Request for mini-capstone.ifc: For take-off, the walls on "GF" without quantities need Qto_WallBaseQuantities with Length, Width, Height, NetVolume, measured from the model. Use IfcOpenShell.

First a look at what the model holds.

```python
import ifcopenshell
import ifcopenshell.util.element
import ifcopenshell.util.unit

model = ifcopenshell.open("mini-capstone.ifc")
print(model.schema)
for unit_type in ("LENGTHUNIT", "AREAUNIT", "VOLUMEUNIT"):
    print(unit_type, ifcopenshell.util.unit.calculate_unit_scale(model, unit_type))
storey = next(s for s in model.by_type("IfcBuildingStorey") if s.Name == "GF")
walls = [e for e in ifcopenshell.util.element.get_decomposition(storey) if e.is_a("IfcWall")]
for e in sorted(walls, key=lambda e: e.id()):
    print(e.id(), e.is_a(), e.Name, list(ifcopenshell.util.element.get_psets(e, qtos_only=True)), sep=" | ")
```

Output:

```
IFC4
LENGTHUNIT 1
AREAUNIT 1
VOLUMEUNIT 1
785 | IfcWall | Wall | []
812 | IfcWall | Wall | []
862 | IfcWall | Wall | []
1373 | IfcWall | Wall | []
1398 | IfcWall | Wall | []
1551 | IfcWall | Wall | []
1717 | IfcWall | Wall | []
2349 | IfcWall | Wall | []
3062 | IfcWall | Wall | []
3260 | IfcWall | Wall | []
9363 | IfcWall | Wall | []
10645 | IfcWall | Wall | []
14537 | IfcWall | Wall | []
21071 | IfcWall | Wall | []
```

```python
import ifcopenshell
import ifcopenshell.api.pset
import ifcopenshell.geom
import ifcopenshell.util.element
import ifcopenshell.util.shape
import ifcopenshell.util.unit

model = ifcopenshell.open("mini-capstone.ifc")
unit_scale = ifcopenshell.util.unit.calculate_unit_scale(model)
volume_scale = ifcopenshell.util.unit.calculate_unit_scale(model, "VOLUMEUNIT")
settings = ifcopenshell.geom.settings()

storey = next(s for s in model.by_type("IfcBuildingStorey") if s.Name == "GF")
walls = [e for e in ifcopenshell.util.element.get_decomposition(storey) if e.is_a("IfcWall")]

for e in sorted(walls, key=lambda e: e.id()):
    if ifcopenshell.util.element.get_psets(e, qtos_only=True, should_inherit=False):
        continue
    # Geometry comes back in metres, in the element's own axes.
    shape = ifcopenshell.geom.create_shape(settings, e)
    values = {
        "Length": ifcopenshell.util.shape.get_x(shape.geometry) / unit_scale,
        "Width": ifcopenshell.util.shape.get_y(shape.geometry) / unit_scale,
        "Height": ifcopenshell.util.shape.get_z(shape.geometry) / unit_scale,
        "NetVolume": ifcopenshell.util.shape.get_volume(shape.geometry) / volume_scale,
    }
    qto = ifcopenshell.api.pset.add_qto(model, product=e, name="Qto_WallBaseQuantities")
    ifcopenshell.api.pset.edit_qto(model, qto=qto, properties=values)
    print(e.id(), {k: round(v, 3) for k, v in values.items()})

model.write("mini-capstone-out.ifc")
```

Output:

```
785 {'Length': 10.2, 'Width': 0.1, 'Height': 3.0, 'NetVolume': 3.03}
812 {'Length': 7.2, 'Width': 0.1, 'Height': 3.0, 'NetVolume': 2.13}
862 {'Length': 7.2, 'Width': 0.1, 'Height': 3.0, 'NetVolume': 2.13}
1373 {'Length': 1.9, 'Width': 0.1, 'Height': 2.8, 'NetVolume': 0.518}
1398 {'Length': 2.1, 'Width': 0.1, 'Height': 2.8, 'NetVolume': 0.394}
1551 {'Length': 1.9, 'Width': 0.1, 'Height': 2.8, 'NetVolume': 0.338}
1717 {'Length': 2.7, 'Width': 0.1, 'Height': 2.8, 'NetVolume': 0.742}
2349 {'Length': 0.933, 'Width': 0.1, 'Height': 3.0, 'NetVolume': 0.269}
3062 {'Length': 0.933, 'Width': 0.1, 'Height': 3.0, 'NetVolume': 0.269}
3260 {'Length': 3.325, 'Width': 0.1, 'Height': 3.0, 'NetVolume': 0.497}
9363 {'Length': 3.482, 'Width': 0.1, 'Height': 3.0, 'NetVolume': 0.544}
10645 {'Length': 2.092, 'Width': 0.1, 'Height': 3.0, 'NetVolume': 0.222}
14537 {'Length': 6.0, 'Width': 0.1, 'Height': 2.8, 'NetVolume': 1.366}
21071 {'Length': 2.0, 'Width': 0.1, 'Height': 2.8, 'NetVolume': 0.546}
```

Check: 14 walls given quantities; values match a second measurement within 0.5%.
